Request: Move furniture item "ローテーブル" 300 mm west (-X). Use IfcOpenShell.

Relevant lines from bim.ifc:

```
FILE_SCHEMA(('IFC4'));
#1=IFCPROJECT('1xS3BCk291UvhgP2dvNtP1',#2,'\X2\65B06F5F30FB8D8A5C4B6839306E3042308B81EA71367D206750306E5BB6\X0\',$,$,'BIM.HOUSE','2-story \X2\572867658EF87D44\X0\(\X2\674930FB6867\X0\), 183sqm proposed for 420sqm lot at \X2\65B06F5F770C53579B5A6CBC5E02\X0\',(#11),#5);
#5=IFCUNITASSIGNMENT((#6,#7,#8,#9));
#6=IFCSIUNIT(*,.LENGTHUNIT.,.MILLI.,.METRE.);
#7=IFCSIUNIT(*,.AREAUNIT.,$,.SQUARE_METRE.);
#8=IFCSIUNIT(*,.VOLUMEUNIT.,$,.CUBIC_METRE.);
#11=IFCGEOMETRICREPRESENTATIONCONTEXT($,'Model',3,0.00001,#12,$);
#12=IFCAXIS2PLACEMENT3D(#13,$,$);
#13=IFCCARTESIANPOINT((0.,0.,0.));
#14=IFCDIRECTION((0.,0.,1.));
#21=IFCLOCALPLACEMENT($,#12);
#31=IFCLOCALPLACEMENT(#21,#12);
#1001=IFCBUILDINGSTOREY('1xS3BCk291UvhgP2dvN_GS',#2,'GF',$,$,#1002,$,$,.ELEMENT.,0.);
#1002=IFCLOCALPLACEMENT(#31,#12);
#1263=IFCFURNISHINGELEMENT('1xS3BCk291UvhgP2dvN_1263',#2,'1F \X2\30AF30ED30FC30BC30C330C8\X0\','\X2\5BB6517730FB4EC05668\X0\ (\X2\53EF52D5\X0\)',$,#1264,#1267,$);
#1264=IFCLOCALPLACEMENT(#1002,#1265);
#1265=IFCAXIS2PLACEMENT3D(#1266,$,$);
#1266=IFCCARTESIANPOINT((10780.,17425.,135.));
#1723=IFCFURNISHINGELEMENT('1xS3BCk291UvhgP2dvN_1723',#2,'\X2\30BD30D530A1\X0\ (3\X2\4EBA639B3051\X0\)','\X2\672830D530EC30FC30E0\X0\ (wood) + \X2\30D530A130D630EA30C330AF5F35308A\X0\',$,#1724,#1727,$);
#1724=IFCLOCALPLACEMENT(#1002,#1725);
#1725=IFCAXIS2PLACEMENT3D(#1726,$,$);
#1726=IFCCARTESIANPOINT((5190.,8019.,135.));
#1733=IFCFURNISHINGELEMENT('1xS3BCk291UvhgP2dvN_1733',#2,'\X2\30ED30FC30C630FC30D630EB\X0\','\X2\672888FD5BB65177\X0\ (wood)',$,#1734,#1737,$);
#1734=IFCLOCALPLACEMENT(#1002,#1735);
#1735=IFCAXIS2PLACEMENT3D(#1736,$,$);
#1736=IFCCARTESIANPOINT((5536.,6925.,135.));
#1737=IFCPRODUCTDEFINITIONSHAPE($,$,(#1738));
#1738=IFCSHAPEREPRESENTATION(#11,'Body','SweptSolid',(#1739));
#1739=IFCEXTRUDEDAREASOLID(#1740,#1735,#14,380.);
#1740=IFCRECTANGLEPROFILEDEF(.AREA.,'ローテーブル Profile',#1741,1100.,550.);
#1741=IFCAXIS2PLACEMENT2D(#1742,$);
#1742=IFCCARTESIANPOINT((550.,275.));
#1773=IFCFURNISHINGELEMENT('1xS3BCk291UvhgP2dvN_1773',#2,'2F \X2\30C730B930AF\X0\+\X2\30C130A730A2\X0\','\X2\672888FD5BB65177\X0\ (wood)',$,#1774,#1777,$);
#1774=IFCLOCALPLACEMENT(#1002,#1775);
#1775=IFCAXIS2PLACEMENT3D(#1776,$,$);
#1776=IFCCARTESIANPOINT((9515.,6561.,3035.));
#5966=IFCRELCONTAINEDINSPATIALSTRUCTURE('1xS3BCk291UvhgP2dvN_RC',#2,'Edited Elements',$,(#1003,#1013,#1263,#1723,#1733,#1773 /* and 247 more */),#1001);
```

```python
import ifcopenshell
import ifcopenshell.api.geometry
import ifcopenshell.util.placement
import ifcopenshell.util.unit

model = ifcopenshell.open("bim.ifc")
unit_scale = ifcopenshell.util.unit.calculate_unit_scale(model)

item = model.by_guid("1xS3BCk291UvhgP2dvN_1733")
matrix = ifcopenshell.util.placement.get_local_placement(item.ObjectPlacement)
matrix[0, 3] -= 0.3 / unit_scale
ifcopenshell.api.geometry.edit_object_placement(model, product=item, matrix=matrix, is_si=False)

print(ifcopenshell.util.placement.get_local_placement(item.ObjectPlacement).round(3) + 0.0)

model.write("bim_edited.ifc")
```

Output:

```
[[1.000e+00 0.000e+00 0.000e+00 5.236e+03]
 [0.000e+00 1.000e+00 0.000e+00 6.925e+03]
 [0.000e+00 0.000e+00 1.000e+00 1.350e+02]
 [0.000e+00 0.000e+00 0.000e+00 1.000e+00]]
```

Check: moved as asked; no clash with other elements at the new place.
